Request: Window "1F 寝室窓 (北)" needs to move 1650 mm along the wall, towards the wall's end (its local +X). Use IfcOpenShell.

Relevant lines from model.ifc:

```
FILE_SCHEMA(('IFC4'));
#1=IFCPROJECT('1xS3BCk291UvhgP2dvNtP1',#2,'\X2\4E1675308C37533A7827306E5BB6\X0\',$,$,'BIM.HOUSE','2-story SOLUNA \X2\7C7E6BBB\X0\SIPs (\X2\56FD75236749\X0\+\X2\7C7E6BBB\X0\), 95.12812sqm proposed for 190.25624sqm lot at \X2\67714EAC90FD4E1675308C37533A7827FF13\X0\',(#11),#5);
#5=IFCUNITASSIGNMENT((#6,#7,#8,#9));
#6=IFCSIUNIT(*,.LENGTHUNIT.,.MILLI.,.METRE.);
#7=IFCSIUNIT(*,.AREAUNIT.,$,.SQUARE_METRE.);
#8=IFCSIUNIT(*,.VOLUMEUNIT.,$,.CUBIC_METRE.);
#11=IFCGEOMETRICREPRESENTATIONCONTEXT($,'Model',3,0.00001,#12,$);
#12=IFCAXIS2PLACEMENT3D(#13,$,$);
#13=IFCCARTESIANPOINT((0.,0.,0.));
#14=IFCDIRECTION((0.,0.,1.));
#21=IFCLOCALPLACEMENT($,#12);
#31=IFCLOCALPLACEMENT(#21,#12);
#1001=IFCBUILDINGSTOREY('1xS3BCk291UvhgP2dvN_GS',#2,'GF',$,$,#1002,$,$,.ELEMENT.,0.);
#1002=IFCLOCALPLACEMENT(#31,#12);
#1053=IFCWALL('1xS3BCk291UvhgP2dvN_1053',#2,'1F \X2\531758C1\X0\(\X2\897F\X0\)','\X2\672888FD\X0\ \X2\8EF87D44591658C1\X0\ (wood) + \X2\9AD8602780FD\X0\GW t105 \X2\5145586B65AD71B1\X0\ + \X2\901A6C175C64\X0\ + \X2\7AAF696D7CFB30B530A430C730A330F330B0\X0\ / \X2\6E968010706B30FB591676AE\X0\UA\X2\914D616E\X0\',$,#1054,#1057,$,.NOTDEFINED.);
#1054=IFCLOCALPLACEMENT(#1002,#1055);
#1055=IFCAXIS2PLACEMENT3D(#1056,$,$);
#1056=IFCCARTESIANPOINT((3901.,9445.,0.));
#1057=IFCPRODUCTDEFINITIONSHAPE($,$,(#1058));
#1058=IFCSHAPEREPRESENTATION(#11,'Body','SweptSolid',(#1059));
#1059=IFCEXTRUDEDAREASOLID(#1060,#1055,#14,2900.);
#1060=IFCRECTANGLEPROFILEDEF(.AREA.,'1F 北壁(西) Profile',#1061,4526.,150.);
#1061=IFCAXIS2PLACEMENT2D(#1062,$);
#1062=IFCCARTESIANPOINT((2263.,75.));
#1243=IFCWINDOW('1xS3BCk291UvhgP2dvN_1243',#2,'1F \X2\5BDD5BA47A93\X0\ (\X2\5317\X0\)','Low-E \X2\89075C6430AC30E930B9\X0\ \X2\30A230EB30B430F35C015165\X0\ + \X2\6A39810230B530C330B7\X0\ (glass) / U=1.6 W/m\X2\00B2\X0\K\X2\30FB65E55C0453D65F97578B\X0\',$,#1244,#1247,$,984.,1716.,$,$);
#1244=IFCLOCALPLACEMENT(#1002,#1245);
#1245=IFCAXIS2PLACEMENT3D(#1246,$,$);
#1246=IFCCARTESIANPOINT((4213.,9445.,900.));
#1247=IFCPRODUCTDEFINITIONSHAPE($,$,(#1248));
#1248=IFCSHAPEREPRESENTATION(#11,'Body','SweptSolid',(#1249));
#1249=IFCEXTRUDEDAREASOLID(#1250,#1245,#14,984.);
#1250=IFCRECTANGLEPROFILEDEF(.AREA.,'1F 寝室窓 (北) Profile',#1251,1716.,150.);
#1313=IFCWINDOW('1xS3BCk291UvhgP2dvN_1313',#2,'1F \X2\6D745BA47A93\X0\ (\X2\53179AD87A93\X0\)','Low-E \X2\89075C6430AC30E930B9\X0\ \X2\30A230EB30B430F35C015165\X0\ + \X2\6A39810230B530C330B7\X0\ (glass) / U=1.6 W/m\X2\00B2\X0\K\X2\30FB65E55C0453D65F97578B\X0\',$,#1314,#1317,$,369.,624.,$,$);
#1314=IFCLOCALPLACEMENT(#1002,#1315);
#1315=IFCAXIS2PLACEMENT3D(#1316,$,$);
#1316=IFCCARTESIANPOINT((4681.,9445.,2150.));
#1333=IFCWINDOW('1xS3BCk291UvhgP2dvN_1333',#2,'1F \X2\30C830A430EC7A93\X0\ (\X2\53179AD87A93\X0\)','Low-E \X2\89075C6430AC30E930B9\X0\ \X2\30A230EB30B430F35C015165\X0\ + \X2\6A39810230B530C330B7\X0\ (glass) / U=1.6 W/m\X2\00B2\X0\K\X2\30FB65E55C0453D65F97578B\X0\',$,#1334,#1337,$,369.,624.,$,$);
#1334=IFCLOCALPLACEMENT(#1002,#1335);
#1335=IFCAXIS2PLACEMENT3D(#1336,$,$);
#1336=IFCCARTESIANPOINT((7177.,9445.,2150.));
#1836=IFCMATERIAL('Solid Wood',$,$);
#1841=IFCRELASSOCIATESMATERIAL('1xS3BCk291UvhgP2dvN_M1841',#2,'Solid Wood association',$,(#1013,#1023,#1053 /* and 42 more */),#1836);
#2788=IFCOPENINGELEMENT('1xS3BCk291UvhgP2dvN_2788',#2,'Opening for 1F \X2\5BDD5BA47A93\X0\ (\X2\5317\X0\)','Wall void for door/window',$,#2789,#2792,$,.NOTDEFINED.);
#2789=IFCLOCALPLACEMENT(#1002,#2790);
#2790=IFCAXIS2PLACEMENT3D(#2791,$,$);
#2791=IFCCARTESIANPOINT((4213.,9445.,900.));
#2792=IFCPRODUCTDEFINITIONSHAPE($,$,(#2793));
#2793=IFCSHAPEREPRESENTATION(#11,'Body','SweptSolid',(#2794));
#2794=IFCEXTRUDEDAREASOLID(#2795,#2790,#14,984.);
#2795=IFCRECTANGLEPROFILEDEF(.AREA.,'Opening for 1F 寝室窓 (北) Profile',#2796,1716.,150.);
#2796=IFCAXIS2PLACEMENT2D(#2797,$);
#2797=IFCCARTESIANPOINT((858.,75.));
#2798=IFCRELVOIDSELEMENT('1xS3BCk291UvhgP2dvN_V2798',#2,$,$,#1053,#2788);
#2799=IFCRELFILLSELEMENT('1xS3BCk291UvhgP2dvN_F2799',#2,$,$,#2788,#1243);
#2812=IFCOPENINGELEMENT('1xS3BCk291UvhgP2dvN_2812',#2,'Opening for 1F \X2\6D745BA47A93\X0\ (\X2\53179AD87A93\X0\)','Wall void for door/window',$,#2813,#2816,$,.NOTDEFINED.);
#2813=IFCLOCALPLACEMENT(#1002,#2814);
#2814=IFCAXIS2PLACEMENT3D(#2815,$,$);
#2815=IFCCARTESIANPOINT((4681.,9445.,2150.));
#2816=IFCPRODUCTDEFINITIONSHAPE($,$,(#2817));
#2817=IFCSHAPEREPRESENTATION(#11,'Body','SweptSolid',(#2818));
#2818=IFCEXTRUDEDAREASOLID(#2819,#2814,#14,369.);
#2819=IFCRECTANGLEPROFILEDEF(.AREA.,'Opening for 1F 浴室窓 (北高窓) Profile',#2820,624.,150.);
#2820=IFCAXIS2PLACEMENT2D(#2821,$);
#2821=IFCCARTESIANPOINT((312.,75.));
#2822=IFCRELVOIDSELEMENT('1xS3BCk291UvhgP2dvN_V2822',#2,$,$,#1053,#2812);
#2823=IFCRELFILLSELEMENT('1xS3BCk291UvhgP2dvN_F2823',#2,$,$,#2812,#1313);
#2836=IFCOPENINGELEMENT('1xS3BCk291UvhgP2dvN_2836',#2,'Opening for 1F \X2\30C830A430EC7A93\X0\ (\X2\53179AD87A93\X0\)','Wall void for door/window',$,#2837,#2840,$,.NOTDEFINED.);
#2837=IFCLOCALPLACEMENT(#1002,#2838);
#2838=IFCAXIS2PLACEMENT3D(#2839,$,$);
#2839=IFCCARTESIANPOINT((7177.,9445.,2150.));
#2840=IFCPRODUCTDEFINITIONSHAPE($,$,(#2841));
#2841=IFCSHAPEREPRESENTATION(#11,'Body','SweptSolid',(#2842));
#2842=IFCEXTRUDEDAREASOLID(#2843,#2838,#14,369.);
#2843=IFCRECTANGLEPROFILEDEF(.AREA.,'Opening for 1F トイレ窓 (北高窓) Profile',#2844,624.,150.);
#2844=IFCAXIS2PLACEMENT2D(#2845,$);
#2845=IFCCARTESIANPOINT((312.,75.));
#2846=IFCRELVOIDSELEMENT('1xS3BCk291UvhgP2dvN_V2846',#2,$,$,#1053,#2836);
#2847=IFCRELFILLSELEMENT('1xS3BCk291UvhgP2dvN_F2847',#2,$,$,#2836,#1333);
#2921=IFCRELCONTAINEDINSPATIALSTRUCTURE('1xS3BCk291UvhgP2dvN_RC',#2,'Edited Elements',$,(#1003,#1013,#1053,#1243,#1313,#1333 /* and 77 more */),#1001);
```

```python
import ifcopenshell
import ifcopenshell.api.geometry
import ifcopenshell.util.placement
import ifcopenshell.util.unit

model = ifcopenshell.open("model.ifc")
unit_scale = ifcopenshell.util.unit.calculate_unit_scale(model)

window = model.by_id(1243)
opening = window.FillsVoids[0].RelatingOpeningElement
wall = opening.VoidsElements[0].RelatingBuildingElement

wall_matrix = ifcopenshell.util.placement.get_local_placement(wall.ObjectPlacement)
shift = wall_matrix[:3, 0] * 1.65 / unit_scale
before = ifcopenshell.util.placement.get_local_placement(window.ObjectPlacement)[:3, 3].copy()

# The window is not placed relative to its opening, so move both.
for product in (opening, window):
    matrix = ifcopenshell.util.placement.get_local_placement(product.ObjectPlacement)
    matrix[:3, 3] += shift
    ifcopenshell.api.geometry.edit_object_placement(model, product=product, matrix=matrix, is_si=False)

after = ifcopenshell.util.placement.get_local_placement(window.ObjectPlacement)[:3, 3]
print("window moved by", (after - before).round(3) + 0.0)

model.write("model_v2.ifc")
```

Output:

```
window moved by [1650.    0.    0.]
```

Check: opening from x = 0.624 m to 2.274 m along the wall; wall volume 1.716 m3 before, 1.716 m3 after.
